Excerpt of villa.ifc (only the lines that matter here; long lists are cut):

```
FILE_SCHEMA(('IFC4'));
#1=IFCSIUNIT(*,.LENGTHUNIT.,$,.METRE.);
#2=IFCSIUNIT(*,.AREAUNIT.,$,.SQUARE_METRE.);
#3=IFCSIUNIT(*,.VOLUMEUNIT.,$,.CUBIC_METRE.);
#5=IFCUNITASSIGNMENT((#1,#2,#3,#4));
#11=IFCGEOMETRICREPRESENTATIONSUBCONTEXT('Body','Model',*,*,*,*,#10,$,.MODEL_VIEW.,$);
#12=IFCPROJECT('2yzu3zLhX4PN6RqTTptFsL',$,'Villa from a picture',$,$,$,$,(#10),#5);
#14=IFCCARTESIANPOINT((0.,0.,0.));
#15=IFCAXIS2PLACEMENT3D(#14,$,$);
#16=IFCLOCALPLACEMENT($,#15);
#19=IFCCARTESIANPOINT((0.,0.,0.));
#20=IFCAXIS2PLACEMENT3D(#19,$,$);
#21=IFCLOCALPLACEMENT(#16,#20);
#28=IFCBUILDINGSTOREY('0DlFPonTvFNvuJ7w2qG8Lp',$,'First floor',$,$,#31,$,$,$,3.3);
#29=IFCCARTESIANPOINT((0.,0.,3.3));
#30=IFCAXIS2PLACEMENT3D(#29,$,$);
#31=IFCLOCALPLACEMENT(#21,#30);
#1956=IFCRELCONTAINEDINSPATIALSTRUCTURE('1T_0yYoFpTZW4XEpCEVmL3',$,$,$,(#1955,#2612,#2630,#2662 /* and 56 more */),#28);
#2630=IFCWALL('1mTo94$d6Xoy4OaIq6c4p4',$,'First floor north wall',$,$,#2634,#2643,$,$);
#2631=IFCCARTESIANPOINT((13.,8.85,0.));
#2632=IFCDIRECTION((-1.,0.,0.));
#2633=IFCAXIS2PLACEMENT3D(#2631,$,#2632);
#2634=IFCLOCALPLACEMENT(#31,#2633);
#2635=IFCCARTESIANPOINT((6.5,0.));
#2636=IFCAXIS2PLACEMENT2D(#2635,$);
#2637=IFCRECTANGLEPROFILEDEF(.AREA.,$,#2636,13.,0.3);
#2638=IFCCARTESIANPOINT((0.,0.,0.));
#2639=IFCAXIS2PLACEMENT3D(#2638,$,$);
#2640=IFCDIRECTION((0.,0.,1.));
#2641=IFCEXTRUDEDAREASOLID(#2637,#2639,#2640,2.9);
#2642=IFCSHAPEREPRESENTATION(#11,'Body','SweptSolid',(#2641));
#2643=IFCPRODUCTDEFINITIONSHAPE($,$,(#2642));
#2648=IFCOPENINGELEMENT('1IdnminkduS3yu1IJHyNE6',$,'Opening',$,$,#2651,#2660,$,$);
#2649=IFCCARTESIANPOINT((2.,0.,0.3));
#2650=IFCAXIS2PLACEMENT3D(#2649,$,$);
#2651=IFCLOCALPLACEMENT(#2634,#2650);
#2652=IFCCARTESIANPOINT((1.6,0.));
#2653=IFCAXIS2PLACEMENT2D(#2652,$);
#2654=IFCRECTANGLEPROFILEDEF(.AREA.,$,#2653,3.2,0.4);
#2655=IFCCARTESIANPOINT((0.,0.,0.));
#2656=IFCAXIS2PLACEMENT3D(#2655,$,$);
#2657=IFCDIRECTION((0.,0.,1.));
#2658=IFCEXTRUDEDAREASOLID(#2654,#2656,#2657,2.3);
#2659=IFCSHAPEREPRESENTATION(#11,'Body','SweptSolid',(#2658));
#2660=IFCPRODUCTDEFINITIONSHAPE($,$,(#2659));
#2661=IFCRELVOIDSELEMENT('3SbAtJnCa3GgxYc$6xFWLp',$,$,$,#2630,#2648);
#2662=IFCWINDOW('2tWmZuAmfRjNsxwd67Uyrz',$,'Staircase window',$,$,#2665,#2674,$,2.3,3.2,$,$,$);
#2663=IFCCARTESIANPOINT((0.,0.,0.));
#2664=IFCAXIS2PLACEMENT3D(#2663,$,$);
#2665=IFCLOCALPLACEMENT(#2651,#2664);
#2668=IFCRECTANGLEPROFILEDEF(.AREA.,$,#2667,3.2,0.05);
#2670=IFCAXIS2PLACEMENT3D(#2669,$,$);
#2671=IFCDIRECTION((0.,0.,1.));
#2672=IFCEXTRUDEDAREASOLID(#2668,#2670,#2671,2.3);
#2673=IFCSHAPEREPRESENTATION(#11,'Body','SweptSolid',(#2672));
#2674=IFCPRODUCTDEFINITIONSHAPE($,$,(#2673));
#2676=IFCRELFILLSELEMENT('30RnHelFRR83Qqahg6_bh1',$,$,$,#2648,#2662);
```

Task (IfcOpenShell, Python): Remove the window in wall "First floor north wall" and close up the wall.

```python
import ifcopenshell
import ifcopenshell.api.feature
import ifcopenshell.api.root
import ifcopenshell.geom
import ifcopenshell.util.shape

model = ifcopenshell.open("villa.ifc")
settings = ifcopenshell.geom.settings()


def volume(element):
    """Net volume in cubic metres, openings subtracted."""
    shape = ifcopenshell.geom.create_shape(settings, element)
    return ifcopenshell.util.shape.get_volume(shape.geometry)


window = model.by_id(2662)
opening = window.FillsVoids[0].RelatingOpeningElement
wall = opening.VoidsElements[0].RelatingBuildingElement
before = volume(wall)

ifcopenshell.api.root.remove_product(model, product=window)
ifcopenshell.api.feature.remove_feature(model, feature=opening)

after = volume(wall)

print(f"wall volume {before:.3f} -> {after:.3f} m3")

model.write("villa_rev.ifc")
```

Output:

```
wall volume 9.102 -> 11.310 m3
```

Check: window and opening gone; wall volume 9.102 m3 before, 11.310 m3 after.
